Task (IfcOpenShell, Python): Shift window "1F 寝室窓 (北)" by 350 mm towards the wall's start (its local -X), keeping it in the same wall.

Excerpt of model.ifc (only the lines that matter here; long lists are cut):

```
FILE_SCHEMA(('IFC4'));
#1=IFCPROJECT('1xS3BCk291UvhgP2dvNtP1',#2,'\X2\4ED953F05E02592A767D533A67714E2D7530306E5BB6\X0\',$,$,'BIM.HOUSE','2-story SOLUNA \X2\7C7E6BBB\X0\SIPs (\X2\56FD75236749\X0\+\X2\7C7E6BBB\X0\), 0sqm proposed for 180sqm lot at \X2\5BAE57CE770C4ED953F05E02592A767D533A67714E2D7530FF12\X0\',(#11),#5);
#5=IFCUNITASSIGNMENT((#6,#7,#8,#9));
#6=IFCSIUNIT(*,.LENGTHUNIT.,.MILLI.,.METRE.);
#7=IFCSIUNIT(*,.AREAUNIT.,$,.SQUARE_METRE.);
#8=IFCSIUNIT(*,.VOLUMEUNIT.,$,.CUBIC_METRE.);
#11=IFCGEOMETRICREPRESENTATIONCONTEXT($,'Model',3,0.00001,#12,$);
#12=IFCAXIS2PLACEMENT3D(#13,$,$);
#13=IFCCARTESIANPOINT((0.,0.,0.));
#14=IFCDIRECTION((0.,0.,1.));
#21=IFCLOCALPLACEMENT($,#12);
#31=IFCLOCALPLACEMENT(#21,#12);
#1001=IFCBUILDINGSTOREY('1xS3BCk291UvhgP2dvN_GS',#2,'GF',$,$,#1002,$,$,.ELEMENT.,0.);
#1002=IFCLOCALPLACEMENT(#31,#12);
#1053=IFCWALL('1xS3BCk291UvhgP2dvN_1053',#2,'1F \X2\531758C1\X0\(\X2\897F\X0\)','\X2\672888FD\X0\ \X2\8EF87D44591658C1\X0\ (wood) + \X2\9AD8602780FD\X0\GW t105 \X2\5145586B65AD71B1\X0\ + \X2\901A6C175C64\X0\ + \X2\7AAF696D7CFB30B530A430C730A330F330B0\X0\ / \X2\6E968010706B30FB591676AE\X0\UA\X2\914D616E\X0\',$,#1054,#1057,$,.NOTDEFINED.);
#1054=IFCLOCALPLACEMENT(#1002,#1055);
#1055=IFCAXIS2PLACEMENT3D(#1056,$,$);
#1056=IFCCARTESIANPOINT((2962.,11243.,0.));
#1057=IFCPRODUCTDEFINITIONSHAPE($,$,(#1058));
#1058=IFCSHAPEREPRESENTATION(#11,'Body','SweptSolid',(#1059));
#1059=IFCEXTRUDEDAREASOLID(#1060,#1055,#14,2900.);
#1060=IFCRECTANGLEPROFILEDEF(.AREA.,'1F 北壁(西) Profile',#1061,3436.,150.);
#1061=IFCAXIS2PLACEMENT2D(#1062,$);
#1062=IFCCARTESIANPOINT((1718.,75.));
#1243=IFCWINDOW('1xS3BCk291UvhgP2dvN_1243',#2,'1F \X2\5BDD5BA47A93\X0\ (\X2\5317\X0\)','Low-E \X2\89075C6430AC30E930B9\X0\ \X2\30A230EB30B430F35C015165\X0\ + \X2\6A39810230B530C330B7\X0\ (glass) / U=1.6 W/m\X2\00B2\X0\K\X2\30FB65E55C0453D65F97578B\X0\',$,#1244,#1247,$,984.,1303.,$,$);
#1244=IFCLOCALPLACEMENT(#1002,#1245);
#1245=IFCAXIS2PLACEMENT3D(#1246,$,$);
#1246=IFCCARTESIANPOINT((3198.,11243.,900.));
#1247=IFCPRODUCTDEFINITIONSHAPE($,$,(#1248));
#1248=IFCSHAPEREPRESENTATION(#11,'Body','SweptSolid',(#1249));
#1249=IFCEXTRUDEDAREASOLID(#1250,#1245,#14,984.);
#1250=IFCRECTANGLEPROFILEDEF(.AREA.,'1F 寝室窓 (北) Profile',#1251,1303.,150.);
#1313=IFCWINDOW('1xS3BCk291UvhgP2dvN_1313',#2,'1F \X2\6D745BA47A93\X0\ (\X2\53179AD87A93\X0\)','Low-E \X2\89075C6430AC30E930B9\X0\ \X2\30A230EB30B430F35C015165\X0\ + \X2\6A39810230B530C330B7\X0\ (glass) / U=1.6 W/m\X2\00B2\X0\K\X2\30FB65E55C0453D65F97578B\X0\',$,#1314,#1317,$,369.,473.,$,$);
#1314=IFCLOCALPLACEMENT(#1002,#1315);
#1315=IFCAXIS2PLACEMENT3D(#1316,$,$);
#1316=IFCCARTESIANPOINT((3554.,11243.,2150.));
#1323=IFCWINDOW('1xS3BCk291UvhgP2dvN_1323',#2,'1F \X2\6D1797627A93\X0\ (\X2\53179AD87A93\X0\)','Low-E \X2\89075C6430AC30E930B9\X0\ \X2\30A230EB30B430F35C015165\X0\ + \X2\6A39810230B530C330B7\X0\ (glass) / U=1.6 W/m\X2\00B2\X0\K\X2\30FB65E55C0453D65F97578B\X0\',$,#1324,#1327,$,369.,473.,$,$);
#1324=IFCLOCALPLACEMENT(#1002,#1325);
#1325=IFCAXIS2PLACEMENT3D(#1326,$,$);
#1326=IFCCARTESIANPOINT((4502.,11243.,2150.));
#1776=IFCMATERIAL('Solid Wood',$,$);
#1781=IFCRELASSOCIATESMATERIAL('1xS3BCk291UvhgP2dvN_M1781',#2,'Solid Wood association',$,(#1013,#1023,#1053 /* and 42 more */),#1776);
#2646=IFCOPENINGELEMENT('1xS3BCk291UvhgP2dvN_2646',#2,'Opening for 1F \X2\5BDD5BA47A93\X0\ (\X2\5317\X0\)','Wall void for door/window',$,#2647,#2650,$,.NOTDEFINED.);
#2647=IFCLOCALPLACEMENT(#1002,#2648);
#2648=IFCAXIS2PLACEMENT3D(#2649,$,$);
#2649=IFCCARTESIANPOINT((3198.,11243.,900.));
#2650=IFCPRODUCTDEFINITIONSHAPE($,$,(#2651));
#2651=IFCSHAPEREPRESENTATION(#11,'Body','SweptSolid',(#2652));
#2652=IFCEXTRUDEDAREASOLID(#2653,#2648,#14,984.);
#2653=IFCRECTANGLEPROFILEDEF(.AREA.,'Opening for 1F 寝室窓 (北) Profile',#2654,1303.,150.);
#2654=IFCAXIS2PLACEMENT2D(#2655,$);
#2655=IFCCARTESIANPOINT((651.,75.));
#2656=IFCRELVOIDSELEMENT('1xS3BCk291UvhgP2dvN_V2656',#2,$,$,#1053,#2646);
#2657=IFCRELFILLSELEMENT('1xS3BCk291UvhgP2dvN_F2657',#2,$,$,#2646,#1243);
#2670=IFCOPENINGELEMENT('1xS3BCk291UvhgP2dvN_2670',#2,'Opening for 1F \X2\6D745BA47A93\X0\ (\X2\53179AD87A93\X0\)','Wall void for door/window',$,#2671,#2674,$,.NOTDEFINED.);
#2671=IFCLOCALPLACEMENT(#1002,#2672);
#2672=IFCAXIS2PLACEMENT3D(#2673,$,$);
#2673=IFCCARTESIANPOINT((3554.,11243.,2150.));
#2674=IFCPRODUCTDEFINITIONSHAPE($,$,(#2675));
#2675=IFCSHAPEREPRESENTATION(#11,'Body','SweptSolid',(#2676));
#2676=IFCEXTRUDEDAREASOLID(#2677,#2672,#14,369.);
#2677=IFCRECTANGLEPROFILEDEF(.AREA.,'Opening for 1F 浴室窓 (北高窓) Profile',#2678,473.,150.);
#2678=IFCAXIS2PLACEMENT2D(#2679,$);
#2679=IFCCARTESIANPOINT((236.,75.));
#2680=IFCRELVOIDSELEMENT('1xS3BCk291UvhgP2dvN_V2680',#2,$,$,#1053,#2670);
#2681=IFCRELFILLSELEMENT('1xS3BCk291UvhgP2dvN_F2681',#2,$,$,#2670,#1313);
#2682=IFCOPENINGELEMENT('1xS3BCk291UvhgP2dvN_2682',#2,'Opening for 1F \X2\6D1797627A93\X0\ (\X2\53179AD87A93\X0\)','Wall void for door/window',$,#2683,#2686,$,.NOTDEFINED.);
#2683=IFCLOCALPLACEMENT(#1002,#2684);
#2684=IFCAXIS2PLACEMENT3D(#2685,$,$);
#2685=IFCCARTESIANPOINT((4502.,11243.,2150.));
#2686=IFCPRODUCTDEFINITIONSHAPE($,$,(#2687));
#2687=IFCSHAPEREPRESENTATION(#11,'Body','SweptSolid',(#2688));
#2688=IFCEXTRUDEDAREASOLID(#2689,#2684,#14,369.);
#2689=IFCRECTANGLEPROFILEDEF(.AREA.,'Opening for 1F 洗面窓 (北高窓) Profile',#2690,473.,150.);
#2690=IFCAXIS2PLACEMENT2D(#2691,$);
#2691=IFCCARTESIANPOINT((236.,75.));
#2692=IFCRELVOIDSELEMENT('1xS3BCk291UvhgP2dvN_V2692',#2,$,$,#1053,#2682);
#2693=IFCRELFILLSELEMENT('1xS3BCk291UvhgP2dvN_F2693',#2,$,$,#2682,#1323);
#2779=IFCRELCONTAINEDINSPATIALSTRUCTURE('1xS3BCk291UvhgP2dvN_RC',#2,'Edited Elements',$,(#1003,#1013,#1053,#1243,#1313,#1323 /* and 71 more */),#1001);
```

```python
import ifcopenshell
import ifcopenshell.api.geometry
import ifcopenshell.util.placement
import ifcopenshell.util.unit

model = ifcopenshell.open("model.ifc")
unit_scale = ifcopenshell.util.unit.calculate_unit_scale(model)

window = model.by_guid("1xS3BCk291UvhgP2dvN_1243")
opening = window.FillsVoids[0].RelatingOpeningElement
wall = opening.VoidsElements[0].RelatingBuildingElement

wall_matrix = ifcopenshell.util.placement.get_local_placement(wall.ObjectPlacement)
shift = wall_matrix[:3, 0] * -0.35 / unit_scale
before = ifcopenshell.util.placement.get_local_placement(window.ObjectPlacement)[:3, 3].copy()

# The window is not placed relative to its opening, so move both.
for product in (opening, window):
    matrix = ifcopenshell.util.placement.get_local_placement(product.ObjectPlacement)
    matrix[:3, 3] += shift
    ifcopenshell.api.geometry.edit_object_placement(model, product=product, matrix=matrix, is_si=False)

after = ifcopenshell.util.placement.get_local_placement(window.ObjectPlacement)[:3, 3]
print("window moved by", (after - before).round(3) + 0.0)

model.write("model-out.ifc")
```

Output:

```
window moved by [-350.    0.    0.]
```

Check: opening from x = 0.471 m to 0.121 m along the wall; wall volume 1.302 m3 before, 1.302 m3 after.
